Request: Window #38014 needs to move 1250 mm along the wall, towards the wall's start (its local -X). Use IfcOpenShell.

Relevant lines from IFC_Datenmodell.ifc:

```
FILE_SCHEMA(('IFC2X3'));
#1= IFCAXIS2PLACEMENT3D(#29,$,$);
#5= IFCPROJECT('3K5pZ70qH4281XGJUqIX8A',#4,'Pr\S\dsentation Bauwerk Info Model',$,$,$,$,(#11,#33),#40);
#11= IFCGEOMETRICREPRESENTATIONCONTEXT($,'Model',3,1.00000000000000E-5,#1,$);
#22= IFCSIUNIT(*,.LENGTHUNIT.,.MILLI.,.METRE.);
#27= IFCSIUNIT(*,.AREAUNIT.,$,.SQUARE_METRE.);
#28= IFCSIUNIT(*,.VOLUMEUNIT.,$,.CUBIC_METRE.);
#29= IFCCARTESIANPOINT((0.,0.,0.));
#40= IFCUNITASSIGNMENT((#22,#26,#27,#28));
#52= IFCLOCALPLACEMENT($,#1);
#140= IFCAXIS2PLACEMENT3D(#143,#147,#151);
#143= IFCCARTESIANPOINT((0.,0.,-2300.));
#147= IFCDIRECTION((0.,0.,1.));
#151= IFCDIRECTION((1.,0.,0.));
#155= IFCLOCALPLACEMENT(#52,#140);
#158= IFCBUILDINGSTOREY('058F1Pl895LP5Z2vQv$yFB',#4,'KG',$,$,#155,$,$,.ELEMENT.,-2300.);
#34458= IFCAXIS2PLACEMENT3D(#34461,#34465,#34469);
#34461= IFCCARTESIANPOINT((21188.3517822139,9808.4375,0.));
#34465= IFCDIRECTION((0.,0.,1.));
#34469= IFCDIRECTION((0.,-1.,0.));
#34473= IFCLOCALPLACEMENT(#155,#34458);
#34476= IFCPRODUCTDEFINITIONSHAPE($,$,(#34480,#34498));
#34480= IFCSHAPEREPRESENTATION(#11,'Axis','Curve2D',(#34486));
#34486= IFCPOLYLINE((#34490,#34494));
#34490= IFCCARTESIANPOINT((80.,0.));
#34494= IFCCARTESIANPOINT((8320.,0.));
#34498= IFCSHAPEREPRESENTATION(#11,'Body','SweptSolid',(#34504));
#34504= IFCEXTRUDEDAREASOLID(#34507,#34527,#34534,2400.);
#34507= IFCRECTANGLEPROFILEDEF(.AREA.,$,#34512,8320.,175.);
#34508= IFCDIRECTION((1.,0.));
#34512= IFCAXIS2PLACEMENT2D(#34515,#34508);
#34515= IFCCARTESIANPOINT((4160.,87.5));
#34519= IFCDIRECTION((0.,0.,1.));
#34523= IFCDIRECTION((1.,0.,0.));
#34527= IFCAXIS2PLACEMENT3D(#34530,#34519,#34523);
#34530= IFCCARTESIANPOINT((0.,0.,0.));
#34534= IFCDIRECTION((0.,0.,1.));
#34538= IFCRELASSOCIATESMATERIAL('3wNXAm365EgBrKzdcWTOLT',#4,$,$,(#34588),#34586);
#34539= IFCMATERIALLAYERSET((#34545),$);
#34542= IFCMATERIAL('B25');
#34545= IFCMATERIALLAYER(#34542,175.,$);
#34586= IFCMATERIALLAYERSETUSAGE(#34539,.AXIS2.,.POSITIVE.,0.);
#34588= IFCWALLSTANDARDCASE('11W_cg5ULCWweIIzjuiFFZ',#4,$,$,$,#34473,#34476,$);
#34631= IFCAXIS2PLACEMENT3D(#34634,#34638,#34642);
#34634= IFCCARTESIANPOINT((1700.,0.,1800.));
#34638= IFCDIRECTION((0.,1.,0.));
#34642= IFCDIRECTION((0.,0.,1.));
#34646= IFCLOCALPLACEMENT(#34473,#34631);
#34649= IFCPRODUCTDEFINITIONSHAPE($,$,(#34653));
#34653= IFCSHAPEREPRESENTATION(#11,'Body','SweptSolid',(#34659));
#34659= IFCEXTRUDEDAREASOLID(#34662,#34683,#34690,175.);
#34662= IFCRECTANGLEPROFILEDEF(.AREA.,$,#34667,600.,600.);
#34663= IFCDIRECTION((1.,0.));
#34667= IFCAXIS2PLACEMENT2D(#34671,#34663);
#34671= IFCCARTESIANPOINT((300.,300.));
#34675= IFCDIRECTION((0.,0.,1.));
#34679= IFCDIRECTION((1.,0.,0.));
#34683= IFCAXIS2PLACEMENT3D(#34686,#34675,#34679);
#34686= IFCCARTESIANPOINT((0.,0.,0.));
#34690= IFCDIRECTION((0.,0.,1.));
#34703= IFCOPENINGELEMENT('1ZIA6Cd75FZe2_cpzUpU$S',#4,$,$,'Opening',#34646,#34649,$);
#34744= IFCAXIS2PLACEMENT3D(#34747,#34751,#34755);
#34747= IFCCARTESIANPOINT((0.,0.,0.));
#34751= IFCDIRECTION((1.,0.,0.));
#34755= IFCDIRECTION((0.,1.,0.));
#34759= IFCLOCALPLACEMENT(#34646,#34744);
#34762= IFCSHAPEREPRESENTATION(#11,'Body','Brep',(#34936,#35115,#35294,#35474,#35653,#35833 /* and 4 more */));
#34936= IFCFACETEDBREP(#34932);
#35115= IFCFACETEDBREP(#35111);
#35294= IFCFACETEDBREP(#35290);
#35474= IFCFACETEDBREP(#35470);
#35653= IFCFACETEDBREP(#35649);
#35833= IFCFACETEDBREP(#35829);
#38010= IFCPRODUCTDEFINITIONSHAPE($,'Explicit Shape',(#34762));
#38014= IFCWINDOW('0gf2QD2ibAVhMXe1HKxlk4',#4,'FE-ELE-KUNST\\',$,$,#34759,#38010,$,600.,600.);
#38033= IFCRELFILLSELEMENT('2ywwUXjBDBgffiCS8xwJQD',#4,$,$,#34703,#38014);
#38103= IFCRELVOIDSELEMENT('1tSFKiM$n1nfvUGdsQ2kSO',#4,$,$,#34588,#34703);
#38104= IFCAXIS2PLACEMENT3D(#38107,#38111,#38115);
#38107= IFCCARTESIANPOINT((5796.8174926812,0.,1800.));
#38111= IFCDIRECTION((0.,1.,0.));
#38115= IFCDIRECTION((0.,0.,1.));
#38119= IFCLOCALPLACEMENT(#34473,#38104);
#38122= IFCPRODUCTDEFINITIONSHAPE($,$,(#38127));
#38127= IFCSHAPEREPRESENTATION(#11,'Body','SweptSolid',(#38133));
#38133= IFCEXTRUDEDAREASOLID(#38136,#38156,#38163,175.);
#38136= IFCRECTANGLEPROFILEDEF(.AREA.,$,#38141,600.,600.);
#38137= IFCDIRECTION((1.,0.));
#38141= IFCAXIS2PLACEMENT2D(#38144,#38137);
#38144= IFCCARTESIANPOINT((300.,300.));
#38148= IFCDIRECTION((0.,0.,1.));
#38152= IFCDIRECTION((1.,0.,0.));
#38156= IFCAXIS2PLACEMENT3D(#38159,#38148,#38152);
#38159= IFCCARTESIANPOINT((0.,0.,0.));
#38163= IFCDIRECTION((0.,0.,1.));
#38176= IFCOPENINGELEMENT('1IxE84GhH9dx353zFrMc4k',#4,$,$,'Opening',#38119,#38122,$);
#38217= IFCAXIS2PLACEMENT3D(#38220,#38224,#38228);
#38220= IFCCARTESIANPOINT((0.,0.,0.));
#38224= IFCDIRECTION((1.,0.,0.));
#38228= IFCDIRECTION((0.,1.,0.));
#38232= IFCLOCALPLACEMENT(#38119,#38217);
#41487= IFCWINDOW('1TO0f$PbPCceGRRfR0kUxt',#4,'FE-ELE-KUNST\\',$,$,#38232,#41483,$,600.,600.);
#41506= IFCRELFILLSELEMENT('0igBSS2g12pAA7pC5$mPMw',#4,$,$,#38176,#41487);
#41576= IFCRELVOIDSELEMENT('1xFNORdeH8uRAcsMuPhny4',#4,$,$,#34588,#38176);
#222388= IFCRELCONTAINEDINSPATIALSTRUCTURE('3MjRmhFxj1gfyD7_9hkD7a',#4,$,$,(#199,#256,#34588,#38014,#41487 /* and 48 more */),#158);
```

```python
import ifcopenshell
import ifcopenshell.api.geometry
import ifcopenshell.util.placement
import ifcopenshell.util.unit

model = ifcopenshell.open("IFC_Datenmodell.ifc")
unit_scale = ifcopenshell.util.unit.calculate_unit_scale(model)

window = model.by_guid("0gf2QD2ibAVhMXe1HKxlk4")
opening = window.FillsVoids[0].RelatingOpeningElement
wall = opening.VoidsElements[0].RelatingBuildingElement

wall_matrix = ifcopenshell.util.placement.get_local_placement(wall.ObjectPlacement)
shift = wall_matrix[:3, 0] * -1.25 / unit_scale
before = ifcopenshell.util.placement.get_local_placement(window.ObjectPlacement)[:3, 3].copy()

# The window is placed relative to its opening, so it follows when the opening moves.
matrix = ifcopenshell.util.placement.get_local_placement(opening.ObjectPlacement)
matrix[:3, 3] += shift
ifcopenshell.api.geometry.edit_object_placement(
    model, product=opening, matrix=matrix, is_si=False, should_transform_children=True
)

after = ifcopenshell.util.placement.get_local_placement(window.ObjectPlacement)[:3, 3]
print("window moved by", (after - before).round(3) + 0.0)

model.write("IFC_Datenmodell_v2.ifc")
```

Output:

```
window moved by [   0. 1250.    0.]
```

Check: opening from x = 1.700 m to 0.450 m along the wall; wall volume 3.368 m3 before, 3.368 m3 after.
